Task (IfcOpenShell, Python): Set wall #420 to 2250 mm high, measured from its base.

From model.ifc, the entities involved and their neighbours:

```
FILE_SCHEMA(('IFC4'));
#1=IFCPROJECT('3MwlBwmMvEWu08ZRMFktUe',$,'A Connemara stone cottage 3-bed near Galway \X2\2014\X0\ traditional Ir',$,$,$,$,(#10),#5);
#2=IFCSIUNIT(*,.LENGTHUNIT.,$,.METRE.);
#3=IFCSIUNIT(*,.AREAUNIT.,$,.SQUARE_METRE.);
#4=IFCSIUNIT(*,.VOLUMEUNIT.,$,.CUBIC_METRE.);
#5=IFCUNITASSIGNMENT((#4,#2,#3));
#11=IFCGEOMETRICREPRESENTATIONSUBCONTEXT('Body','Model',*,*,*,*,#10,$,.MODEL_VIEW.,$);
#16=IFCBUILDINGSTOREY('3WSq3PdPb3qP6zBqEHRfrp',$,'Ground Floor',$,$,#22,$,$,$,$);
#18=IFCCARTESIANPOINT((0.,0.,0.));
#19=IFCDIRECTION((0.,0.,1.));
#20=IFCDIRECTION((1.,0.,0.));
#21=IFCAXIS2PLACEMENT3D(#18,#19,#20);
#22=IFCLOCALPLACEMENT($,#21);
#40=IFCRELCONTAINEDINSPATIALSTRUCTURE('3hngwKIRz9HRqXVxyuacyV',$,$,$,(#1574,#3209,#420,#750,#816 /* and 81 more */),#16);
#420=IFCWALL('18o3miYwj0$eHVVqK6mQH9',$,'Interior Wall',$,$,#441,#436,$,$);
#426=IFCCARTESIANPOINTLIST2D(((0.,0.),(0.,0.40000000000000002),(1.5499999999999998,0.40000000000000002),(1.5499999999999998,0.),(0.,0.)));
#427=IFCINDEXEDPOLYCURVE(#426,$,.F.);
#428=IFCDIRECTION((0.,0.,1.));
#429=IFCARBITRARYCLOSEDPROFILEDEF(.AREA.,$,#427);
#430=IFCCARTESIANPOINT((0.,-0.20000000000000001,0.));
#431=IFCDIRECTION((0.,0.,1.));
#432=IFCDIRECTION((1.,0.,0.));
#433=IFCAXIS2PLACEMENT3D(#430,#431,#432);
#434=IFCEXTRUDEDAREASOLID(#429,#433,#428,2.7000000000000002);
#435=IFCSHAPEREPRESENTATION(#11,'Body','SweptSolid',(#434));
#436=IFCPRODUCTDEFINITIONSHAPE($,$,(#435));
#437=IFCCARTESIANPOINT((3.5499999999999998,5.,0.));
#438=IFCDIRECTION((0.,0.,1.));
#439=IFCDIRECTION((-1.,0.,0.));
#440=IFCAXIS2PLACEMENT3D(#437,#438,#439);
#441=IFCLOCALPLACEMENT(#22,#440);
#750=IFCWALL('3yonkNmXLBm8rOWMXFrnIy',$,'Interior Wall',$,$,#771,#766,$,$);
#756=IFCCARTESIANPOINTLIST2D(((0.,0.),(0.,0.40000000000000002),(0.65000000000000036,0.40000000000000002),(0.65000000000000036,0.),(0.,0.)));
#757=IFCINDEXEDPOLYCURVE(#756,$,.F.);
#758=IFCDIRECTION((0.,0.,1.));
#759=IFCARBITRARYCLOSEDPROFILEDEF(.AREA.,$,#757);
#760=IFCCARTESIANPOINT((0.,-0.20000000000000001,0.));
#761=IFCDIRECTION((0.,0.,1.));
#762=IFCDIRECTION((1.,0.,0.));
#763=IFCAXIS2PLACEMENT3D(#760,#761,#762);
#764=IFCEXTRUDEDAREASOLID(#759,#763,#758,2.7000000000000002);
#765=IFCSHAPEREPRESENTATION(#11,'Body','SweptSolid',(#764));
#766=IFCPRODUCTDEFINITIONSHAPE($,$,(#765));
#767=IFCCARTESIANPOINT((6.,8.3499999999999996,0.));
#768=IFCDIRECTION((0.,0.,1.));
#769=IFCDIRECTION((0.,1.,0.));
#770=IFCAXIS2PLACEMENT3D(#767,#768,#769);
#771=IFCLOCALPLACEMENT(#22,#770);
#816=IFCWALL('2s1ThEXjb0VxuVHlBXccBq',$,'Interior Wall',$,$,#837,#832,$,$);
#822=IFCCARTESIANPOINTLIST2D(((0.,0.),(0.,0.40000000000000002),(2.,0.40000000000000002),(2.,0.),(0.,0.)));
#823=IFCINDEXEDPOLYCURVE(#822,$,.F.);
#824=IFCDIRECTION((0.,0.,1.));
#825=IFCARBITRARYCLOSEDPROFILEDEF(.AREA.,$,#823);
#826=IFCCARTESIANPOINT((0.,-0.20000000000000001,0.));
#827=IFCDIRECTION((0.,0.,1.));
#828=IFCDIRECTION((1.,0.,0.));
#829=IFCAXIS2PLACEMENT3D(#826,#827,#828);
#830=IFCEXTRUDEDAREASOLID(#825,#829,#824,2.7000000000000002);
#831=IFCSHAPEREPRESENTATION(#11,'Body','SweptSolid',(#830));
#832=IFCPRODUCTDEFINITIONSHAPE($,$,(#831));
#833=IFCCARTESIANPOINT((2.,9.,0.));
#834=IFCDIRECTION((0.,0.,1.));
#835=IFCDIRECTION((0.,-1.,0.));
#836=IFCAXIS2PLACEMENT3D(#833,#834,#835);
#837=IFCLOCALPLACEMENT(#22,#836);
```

```python
import ifcopenshell
import ifcopenshell.geom
import ifcopenshell.util.representation
import ifcopenshell.util.shape

model = ifcopenshell.open("model.ifc")
settings = ifcopenshell.geom.settings()


def volume(element):
    """Net volume in cubic metres, openings subtracted."""
    shape = ifcopenshell.geom.create_shape(settings, element)
    return ifcopenshell.util.shape.get_volume(shape.geometry)


wall = model.by_guid("18o3miYwj0$eHVVqK6mQH9")
before = volume(wall)

body = ifcopenshell.util.representation.get_representation(wall, "Model", "Body")
solid = body.Items[0]
old_height = solid.Depth
solid.Depth = 2.25
after = volume(wall)

print(f"height {old_height:g} -> {solid.Depth:g}, volume {before:.3f} -> {after:.3f} m3")

model.write("model_updated.ifc")
```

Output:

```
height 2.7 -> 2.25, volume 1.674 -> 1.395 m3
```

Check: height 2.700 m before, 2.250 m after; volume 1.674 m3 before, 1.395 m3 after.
